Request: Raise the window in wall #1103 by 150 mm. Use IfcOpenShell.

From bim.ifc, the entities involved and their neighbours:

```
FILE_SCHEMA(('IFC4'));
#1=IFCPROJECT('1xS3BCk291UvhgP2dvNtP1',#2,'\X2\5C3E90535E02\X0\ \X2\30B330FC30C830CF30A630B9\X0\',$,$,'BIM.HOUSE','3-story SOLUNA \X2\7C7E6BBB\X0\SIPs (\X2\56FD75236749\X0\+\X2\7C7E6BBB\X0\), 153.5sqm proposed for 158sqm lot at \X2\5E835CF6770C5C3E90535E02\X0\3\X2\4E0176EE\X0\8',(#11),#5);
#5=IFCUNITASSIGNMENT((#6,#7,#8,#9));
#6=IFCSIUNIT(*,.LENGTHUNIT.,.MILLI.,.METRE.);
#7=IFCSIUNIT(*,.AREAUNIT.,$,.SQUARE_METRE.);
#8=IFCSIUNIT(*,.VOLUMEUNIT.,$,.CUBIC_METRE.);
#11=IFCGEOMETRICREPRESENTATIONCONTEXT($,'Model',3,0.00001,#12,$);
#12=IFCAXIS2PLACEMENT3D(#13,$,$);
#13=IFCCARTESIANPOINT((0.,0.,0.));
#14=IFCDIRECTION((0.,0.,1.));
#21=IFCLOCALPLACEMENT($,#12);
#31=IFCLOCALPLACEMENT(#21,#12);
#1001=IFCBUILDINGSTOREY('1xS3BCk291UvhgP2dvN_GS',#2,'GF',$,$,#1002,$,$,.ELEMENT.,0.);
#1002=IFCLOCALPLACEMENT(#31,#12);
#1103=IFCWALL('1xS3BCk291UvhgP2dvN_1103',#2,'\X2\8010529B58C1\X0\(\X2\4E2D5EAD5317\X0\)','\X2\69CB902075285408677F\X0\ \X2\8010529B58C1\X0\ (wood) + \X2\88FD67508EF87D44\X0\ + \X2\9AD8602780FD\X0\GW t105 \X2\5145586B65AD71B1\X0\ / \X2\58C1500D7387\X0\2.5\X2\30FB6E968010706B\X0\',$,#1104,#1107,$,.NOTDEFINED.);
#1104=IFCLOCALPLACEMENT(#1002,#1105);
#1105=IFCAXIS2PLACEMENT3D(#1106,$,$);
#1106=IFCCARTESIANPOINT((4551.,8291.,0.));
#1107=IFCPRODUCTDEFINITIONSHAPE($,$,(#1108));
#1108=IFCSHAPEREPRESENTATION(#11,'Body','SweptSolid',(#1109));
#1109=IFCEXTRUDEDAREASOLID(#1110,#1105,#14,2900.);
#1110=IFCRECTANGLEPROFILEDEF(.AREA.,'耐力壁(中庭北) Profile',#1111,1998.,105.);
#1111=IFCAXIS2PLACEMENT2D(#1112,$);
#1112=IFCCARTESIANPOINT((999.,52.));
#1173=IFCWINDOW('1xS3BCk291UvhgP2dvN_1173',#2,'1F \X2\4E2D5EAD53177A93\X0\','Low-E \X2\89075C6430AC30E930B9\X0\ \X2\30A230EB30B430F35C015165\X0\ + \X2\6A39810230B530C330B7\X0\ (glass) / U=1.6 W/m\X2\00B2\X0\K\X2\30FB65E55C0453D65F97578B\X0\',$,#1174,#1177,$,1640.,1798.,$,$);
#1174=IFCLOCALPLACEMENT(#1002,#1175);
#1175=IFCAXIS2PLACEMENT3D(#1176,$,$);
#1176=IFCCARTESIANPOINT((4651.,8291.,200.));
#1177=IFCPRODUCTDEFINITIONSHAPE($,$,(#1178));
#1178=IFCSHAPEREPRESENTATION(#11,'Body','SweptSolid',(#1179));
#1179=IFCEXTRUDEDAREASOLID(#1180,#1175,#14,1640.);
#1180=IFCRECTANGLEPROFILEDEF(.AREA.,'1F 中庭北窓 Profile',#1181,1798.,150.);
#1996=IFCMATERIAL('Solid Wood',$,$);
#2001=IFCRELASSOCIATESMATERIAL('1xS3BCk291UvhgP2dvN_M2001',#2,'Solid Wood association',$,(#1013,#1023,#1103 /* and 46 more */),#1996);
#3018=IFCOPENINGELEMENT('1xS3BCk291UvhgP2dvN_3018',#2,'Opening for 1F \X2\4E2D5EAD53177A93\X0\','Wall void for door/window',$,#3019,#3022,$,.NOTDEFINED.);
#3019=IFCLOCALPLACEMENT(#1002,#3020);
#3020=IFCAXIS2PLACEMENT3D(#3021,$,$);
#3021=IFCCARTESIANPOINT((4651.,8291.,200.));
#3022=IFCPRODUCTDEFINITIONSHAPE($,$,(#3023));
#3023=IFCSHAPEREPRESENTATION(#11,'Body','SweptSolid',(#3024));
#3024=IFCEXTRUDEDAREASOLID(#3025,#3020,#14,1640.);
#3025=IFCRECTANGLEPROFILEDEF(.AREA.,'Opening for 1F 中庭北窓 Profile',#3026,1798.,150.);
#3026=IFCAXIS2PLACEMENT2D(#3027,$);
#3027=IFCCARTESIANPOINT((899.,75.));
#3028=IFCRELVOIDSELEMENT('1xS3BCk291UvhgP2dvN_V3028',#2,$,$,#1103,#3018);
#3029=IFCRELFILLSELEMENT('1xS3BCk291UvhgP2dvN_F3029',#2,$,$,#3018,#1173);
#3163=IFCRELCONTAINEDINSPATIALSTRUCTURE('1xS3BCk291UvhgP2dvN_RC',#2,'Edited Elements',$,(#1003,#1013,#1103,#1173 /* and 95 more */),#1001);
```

```python
import numpy as np
import ifcopenshell
import ifcopenshell.api.geometry
import ifcopenshell.util.placement
import ifcopenshell.util.unit

model = ifcopenshell.open("bim.ifc")
unit_scale = ifcopenshell.util.unit.calculate_unit_scale(model)

window = model.by_guid("1xS3BCk291UvhgP2dvN_1173")
opening = window.FillsVoids[0].RelatingOpeningElement
dz = 150.0

shift = np.array([0.0, 0.0, dz])
# The window is not placed relative to its opening, so move both.
for product in (opening, window):
    matrix = ifcopenshell.util.placement.get_local_placement(product.ObjectPlacement)
    matrix[:3, 3] += shift
    ifcopenshell.api.geometry.edit_object_placement(model, product=product, matrix=matrix, is_si=False)

print(f"moved by {dz * unit_scale:+.3f} m")

model.write("bim-out.ifc")
```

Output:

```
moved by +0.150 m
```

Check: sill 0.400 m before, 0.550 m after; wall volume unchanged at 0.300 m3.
